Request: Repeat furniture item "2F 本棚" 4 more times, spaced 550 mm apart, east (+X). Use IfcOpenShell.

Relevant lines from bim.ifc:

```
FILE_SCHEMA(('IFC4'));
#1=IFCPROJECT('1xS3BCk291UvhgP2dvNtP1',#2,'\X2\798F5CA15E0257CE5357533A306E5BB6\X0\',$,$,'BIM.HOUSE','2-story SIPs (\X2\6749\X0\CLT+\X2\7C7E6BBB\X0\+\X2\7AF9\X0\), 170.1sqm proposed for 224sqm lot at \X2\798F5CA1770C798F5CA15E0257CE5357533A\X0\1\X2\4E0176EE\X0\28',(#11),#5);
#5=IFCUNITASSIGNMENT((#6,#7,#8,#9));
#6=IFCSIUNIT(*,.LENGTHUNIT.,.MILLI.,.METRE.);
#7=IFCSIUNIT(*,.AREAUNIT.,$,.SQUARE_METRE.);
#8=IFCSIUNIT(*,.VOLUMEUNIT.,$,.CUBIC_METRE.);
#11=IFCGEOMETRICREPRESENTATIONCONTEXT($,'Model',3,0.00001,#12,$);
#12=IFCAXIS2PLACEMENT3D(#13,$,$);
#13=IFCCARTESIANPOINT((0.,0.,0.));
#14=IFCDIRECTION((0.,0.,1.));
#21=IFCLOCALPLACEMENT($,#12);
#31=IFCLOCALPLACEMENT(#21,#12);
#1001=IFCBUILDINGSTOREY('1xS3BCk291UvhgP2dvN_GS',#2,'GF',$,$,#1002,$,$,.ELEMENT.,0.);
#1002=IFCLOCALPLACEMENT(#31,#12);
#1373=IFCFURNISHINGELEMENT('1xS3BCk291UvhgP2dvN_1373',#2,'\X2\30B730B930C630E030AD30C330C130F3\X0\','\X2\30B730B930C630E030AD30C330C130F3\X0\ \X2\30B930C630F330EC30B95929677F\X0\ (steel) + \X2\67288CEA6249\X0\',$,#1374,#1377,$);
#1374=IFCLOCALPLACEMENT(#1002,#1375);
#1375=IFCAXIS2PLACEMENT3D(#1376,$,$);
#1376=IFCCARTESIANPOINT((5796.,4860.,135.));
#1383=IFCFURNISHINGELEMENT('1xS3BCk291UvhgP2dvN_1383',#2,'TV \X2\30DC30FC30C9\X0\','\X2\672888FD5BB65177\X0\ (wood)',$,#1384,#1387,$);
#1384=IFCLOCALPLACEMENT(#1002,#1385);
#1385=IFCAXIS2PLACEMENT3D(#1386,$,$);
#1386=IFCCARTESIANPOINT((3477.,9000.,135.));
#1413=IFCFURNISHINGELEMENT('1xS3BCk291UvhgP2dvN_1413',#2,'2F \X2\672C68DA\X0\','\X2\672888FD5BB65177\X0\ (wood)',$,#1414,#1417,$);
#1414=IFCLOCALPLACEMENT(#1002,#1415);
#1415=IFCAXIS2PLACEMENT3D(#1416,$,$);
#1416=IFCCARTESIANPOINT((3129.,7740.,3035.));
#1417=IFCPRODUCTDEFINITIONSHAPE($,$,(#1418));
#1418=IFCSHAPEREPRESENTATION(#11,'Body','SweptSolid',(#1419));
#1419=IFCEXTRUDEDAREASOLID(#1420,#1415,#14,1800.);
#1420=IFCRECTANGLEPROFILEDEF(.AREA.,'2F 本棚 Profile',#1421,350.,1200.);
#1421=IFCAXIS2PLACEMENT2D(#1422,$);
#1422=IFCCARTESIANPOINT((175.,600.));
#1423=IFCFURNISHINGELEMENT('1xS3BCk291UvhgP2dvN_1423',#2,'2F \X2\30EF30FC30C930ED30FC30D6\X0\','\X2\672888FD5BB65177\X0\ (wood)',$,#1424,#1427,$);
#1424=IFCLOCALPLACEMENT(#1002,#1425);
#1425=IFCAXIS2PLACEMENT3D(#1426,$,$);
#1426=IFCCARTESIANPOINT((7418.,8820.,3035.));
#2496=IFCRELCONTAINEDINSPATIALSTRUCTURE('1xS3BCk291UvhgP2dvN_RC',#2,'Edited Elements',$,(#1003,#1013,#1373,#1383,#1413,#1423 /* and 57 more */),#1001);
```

```python
import numpy as np
import ifcopenshell
import ifcopenshell.api.geometry
import ifcopenshell.api.root
import ifcopenshell.util.element
import ifcopenshell.util.placement

model = ifcopenshell.open("bim.ifc")


def reuse_history(source, copy):
    """copy_class also copies each property set's owner history, people and application; keep the originals."""
    for rel in copy.IsDefinedBy:
        if rel.is_a("IfcRelDefinesByProperties") and (history := rel.RelatingPropertyDefinition.OwnerHistory):
            rel.RelatingPropertyDefinition.OwnerHistory = source.OwnerHistory
            ifcopenshell.util.element.remove_deep2(model, history)


source = model.by_guid("1xS3BCk291UvhgP2dvN_1413")
base = ifcopenshell.util.placement.get_local_placement(source.ObjectPlacement)
step = np.array([1.0, 0.0, 0.0]) * 550.0

for i in range(1, 5):
    copy = ifcopenshell.api.root.copy_class(model, product=source)
    copy.Representation = ifcopenshell.util.element.copy_deep(
        model, source.Representation, exclude=["IfcGeometricRepresentationContext", "IfcRepresentationMap"]
    )
    reuse_history(source, copy)
    matrix = base.copy()
    matrix[:3, 3] += i * step
    print("added at", matrix[:3, 3].round(3) + 0.0)
    ifcopenshell.api.geometry.edit_object_placement(model, product=copy, matrix=matrix, is_si=False)

model.write("bim-out.ifc")
```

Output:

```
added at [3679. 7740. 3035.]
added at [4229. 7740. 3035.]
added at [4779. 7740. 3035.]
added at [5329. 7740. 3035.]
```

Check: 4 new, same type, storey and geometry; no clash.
